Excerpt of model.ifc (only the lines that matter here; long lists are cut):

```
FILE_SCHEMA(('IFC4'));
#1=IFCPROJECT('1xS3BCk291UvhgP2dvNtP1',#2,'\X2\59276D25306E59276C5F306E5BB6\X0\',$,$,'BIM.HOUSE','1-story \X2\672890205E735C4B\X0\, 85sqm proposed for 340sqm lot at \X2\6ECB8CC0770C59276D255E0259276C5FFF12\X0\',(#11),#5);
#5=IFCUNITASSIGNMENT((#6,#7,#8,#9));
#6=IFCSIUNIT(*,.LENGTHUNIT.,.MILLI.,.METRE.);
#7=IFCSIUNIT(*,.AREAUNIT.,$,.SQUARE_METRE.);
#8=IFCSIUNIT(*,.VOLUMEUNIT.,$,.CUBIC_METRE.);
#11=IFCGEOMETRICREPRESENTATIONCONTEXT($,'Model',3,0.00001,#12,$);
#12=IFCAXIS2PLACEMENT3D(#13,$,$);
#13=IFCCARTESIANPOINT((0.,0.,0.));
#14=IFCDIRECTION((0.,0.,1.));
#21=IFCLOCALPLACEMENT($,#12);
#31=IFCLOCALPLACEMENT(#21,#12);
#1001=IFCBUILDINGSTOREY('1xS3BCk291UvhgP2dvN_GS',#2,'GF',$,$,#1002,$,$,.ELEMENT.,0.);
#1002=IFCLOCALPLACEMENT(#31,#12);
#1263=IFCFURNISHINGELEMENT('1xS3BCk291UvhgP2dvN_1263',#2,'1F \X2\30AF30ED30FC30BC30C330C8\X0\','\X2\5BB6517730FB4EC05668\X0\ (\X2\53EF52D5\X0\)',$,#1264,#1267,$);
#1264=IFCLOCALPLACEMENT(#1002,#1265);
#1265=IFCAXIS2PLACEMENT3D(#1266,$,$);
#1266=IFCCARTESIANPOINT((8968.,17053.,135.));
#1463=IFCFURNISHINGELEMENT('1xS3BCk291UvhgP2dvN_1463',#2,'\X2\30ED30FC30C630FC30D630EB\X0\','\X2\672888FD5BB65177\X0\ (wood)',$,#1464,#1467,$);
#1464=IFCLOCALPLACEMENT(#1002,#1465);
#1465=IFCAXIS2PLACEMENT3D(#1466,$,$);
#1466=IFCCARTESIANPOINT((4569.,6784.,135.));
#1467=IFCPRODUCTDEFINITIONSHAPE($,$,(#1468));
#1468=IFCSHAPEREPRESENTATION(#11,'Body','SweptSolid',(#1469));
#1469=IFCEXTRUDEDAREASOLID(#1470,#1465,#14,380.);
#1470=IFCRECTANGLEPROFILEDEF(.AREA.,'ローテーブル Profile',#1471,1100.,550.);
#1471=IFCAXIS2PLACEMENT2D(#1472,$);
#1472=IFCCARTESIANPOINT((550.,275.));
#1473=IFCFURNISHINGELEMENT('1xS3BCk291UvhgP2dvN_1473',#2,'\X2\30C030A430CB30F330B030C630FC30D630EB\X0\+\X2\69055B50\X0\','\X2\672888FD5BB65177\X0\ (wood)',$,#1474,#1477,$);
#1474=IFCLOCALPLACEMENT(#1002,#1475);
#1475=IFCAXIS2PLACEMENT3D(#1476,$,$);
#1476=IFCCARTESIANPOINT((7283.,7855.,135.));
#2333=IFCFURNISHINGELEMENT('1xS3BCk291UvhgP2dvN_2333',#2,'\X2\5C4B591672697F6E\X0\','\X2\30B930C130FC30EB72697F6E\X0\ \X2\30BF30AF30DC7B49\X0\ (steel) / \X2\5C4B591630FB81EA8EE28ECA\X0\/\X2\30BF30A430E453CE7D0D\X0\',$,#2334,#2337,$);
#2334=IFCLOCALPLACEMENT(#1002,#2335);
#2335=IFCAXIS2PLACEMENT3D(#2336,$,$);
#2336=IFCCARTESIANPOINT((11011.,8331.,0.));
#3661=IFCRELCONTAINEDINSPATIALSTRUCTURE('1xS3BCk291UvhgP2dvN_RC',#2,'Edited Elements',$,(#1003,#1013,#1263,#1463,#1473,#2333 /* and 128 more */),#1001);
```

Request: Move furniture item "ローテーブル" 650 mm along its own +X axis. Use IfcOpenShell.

```python
import ifcopenshell
import ifcopenshell.api.geometry
import ifcopenshell.util.placement
import ifcopenshell.util.unit

model = ifcopenshell.open("model.ifc")
unit_scale = ifcopenshell.util.unit.calculate_unit_scale(model)

item = model.by_guid("1xS3BCk291UvhgP2dvN_1463")
matrix = ifcopenshell.util.placement.get_local_placement(item.ObjectPlacement)
matrix[:3, 3] += matrix[:3, 0] * 0.65 / unit_scale
ifcopenshell.api.geometry.edit_object_placement(model, product=item, matrix=matrix, is_si=False)

print(ifcopenshell.util.placement.get_local_placement(item.ObjectPlacement).round(3) + 0.0)

model.write("model_edited.ifc")
```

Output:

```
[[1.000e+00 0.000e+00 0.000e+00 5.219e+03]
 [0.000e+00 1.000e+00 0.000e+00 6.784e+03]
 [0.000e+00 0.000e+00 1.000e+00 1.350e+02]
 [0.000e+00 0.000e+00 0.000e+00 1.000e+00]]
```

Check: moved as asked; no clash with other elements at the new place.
